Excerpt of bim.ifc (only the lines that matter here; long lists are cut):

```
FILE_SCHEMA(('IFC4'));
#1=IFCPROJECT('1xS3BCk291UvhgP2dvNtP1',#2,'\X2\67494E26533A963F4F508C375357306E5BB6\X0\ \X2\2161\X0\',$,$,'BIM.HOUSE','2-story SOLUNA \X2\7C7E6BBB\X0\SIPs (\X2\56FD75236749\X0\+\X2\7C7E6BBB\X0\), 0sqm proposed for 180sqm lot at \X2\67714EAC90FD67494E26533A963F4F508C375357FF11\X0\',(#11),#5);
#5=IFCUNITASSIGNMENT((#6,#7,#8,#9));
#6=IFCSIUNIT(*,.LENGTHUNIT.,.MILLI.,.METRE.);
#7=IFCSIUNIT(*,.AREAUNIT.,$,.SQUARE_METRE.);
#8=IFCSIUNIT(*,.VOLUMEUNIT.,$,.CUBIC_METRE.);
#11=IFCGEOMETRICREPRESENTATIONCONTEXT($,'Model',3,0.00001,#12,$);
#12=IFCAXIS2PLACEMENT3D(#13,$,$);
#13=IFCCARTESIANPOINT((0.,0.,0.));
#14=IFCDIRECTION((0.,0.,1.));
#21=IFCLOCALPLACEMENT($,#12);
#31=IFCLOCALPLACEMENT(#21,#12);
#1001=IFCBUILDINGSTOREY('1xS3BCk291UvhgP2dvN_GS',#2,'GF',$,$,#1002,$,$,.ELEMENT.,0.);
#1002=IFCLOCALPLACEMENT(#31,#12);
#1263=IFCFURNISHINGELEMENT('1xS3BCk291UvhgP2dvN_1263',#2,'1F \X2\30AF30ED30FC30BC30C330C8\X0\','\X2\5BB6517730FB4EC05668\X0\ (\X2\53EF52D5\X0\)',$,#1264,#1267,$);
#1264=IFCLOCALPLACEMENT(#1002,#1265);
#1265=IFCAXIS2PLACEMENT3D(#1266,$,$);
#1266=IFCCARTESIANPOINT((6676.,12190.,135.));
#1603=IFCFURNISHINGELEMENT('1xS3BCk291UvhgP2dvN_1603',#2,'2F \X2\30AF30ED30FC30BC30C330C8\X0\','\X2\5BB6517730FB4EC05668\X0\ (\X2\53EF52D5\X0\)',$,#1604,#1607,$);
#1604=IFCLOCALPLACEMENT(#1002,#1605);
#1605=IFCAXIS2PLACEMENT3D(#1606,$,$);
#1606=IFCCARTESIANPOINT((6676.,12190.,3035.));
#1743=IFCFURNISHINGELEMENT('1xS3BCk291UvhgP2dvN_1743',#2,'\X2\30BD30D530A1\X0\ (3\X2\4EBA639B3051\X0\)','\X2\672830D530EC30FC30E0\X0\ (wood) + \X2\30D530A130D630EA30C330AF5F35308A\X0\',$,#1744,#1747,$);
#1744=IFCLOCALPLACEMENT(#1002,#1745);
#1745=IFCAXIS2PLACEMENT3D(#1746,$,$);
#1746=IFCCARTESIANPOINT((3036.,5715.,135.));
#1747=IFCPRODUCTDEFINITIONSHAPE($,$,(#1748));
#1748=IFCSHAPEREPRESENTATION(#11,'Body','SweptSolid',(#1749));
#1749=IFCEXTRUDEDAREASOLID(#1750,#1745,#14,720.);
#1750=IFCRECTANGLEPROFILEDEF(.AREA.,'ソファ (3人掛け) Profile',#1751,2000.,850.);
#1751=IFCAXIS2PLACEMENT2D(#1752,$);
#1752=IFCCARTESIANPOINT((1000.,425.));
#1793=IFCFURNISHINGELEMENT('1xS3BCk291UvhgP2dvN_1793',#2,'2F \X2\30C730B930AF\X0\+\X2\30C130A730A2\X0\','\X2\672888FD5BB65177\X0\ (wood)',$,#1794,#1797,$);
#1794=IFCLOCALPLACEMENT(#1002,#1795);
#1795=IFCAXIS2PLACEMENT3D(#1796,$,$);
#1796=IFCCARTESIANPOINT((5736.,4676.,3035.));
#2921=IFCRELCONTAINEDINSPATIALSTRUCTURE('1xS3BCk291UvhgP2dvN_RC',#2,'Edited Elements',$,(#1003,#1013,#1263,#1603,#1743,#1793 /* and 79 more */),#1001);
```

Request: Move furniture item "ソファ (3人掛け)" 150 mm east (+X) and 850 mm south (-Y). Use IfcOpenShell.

```python
import ifcopenshell
import ifcopenshell.api.geometry
import ifcopenshell.util.placement

model = ifcopenshell.open("bim.ifc")

item = model.by_guid("1xS3BCk291UvhgP2dvN_1743")
matrix = ifcopenshell.util.placement.get_local_placement(item.ObjectPlacement)
matrix[0, 3] += 150.0
matrix[1, 3] -= 850.0
ifcopenshell.api.geometry.edit_object_placement(model, product=item, matrix=matrix, is_si=False)

print(ifcopenshell.util.placement.get_local_placement(item.ObjectPlacement).round(3) + 0.0)

model.write("bim_v2.ifc")
```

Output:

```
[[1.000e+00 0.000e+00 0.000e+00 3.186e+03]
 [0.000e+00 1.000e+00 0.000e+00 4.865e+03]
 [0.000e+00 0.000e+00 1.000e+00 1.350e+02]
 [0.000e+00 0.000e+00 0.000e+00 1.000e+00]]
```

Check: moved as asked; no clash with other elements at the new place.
